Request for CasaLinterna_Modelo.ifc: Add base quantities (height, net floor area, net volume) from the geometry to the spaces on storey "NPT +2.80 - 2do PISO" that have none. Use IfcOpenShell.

First a look at what the model holds.

```python
import ifcopenshell
import ifcopenshell.util.element
import ifcopenshell.util.unit

model = ifcopenshell.open("CasaLinterna_Modelo.ifc")
print(model.schema)
for unit_type in ("LENGTHUNIT", "AREAUNIT", "VOLUMEUNIT"):
    print(unit_type, ifcopenshell.util.unit.calculate_unit_scale(model, unit_type))
storey = next(s for s in model.by_type("IfcBuildingStorey") if s.Name == "NPT +2.80 - 2do PISO")
spaces = [e for e in ifcopenshell.util.element.get_decomposition(storey) if e.is_a("IfcSpace")]
for e in sorted(spaces, key=lambda e: e.id()):
    print(e.id(), e.is_a(), e.Name, list(ifcopenshell.util.element.get_psets(e, qtos_only=True)), sep=" | ")
```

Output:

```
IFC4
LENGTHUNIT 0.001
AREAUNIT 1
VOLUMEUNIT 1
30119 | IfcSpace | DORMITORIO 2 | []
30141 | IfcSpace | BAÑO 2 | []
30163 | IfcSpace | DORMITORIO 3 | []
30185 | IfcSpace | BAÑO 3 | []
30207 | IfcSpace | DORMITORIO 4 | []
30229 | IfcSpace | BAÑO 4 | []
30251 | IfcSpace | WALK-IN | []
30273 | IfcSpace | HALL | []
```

```python
import ifcopenshell
import ifcopenshell.api.pset
import ifcopenshell.geom
import ifcopenshell.util.element
import ifcopenshell.util.shape
import ifcopenshell.util.unit

model = ifcopenshell.open("CasaLinterna_Modelo.ifc")
unit_scale = ifcopenshell.util.unit.calculate_unit_scale(model)
area_scale = ifcopenshell.util.unit.calculate_unit_scale(model, "AREAUNIT")
volume_scale = ifcopenshell.util.unit.calculate_unit_scale(model, "VOLUMEUNIT")
settings = ifcopenshell.geom.settings()

storey = next(s for s in model.by_type("IfcBuildingStorey") if s.Name == "NPT +2.80 - 2do PISO")
spaces = [e for e in ifcopenshell.util.element.get_decomposition(storey) if e.is_a("IfcSpace")]

for e in sorted(spaces, key=lambda e: e.id()):
    if ifcopenshell.util.element.get_psets(e, qtos_only=True, should_inherit=False):
        continue
    # Geometry comes back in metres, in the element's own axes.
    shape = ifcopenshell.geom.create_shape(settings, e)
    values = {
        "Height": ifcopenshell.util.shape.get_z(shape.geometry) / unit_scale,
        "NetFloorArea": ifcopenshell.util.shape.get_footprint_area(shape.geometry) / area_scale,
        "NetVolume": ifcopenshell.util.shape.get_volume(shape.geometry) / volume_scale,
    }
    qto = ifcopenshell.api.pset.add_qto(model, product=e, name="Qto_SpaceBaseQuantities")
    ifcopenshell.api.pset.edit_qto(model, qto=qto, properties=values)
    print(e.id(), {k: round(v, 3) for k, v in values.items()})

model.write("CasaLinterna_Modelo_rev.ifc")
```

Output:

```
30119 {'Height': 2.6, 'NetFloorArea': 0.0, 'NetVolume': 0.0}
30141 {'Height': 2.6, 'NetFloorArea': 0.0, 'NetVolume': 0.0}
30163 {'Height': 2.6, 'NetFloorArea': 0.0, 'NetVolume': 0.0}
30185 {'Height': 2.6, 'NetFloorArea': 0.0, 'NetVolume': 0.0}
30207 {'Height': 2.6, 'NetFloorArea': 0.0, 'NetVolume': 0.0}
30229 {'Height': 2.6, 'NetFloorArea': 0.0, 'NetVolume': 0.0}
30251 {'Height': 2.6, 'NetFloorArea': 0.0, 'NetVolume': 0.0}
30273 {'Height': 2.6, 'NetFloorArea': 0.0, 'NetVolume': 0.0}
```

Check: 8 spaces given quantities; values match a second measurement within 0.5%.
